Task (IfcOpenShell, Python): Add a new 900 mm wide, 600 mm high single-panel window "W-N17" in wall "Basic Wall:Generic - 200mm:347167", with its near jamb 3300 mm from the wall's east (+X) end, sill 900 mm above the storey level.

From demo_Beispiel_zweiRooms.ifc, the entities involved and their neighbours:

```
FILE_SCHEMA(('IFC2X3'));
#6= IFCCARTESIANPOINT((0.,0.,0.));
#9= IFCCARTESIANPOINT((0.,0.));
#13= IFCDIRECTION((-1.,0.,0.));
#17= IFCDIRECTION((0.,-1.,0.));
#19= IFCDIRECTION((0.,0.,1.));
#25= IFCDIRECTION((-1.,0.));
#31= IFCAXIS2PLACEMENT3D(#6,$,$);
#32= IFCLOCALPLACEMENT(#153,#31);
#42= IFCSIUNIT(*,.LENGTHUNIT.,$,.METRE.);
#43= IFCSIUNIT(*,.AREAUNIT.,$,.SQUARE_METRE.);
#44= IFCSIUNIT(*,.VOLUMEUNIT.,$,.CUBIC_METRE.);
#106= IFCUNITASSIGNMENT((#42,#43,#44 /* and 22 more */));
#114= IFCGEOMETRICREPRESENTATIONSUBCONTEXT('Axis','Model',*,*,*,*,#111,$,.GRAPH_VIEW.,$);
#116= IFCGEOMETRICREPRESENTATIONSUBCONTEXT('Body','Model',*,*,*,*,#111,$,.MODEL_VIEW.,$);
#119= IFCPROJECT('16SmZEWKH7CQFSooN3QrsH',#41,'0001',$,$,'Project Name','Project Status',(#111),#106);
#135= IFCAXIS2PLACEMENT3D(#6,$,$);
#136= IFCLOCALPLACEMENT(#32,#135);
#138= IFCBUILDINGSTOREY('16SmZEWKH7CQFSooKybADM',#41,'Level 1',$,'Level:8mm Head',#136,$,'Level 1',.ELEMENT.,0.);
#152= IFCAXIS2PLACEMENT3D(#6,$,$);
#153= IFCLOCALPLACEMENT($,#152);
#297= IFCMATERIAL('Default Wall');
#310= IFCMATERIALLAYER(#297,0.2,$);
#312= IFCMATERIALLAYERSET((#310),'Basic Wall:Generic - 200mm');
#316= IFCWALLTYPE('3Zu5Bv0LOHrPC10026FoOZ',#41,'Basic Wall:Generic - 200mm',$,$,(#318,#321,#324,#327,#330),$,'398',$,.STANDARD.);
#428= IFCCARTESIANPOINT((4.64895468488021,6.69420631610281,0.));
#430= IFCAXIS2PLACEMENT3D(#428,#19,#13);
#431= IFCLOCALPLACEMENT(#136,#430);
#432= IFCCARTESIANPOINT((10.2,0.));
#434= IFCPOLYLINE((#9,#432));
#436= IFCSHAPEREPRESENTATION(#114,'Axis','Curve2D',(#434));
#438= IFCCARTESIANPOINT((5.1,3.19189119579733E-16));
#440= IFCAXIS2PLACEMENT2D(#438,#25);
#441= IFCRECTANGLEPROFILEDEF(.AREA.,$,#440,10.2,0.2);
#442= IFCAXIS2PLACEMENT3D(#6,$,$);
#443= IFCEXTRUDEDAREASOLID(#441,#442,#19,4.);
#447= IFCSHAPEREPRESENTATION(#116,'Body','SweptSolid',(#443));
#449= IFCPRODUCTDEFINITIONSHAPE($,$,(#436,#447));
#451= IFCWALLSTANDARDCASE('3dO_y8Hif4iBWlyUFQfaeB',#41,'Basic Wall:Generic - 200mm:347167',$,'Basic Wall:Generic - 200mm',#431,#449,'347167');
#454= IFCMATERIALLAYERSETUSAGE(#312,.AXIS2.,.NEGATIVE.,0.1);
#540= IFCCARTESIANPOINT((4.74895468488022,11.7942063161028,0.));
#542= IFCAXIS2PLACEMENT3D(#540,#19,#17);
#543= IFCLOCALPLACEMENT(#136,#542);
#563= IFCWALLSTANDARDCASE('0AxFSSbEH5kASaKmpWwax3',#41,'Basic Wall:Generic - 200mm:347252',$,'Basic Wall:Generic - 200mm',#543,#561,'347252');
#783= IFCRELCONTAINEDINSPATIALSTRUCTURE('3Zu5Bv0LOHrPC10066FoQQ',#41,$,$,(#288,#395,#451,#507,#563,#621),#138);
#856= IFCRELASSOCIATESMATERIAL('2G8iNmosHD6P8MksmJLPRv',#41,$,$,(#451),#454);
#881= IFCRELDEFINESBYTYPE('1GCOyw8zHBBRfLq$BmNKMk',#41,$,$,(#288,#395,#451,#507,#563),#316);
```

```python
import numpy as np
import ifcopenshell
import ifcopenshell.api.feature
import ifcopenshell.api.geometry
import ifcopenshell.api.root
import ifcopenshell.api.spatial
import ifcopenshell.api.type
import ifcopenshell.geom
import ifcopenshell.util.element
import ifcopenshell.util.placement
import ifcopenshell.util.representation
import ifcopenshell.util.shape
import ifcopenshell.util.unit

model = ifcopenshell.open("demo_Beispiel_zweiRooms.ifc")
unit_scale = ifcopenshell.util.unit.calculate_unit_scale(model)
settings = ifcopenshell.geom.settings()


def volume(element):
    """Net volume in cubic metres, openings subtracted."""
    shape = ifcopenshell.geom.create_shape(settings, element)
    return ifcopenshell.util.shape.get_volume(shape.geometry)


wall = model.by_id(451)
storey = ifcopenshell.util.element.get_container(wall, ifc_class="IfcBuildingStorey")
context = ifcopenshell.util.representation.get_context(model, "Model", "Body", "MODEL_VIEW")
before = volume(wall)

width, height, from_end, sill = 0.9, 0.6, 3.3, 0.9  # metres

# The wall runs along its own X axis, and the end named is its -X end.
wall_shape = ifcopenshell.geom.create_shape(settings, wall)
x, y, z = ifcopenshell.util.shape.get_vertices(wall_shape.geometry).T
start = x.min() + from_end
face, thickness = float(y.min()), float(y.max() - y.min())
wall_matrix = ifcopenshell.util.placement.get_local_placement(wall.ObjectPlacement)
level = ifcopenshell.util.placement.get_local_placement(storey.ObjectPlacement)[2, 3]


def in_wall(x, y):
    """Placement at x, y metres in the wall's axes, at sill height."""
    matrix = wall_matrix.copy()
    matrix[:, 3] = wall_matrix @ np.array([x / unit_scale, y / unit_scale, 0.0, 1.0])
    matrix[2, 3] = level + sill / unit_scale
    return matrix


# Opening: a box that overshoots both wall faces by 50 mm.
opening = ifcopenshell.api.root.create_entity(model, ifc_class="IfcOpeningElement")
box = ifcopenshell.api.geometry.add_wall_representation(
    model, context=context, length=width, height=height, thickness=thickness + 0.1
)
ifcopenshell.api.geometry.assign_representation(model, product=opening, representation=box)
ifcopenshell.api.geometry.edit_object_placement(model, product=opening, matrix=in_wall(start, face - 0.05), is_si=False)
ifcopenshell.api.feature.add_feature(model, feature=opening, element=wall)

window = ifcopenshell.api.root.create_entity(model, ifc_class="IfcWindow", name="W-N17")
window.OverallWidth, window.OverallHeight = width / unit_scale, height / unit_scale
body = ifcopenshell.api.geometry.add_window_representation(
    model,
    context=context,
    overall_width=window.OverallWidth,
    overall_height=window.OverallHeight,
    partition_type="SINGLE_PANEL",
)
ifcopenshell.api.geometry.assign_representation(model, product=window, representation=body)
ifcopenshell.api.spatial.assign_container(model, products=[window], relating_structure=storey)
fills = ifcopenshell.api.feature.add_filling(model, opening=opening, element=window)
fills.OwnerHistory = window.OwnerHistory  # required in IFC2X3

# IFC2X3 keeps the operation on the window style.
style = ifcopenshell.api.root.create_entity(model, ifc_class="IfcWindowStyle", name="W-N17")
style.OperationType, style.ConstructionType = "SINGLE_PANEL", "NOTDEFINED"
style.ParameterTakesPrecedence = style.Sizeable = False
ifcopenshell.api.type.assign_type(model, related_objects=[window], relating_type=style)

# Centre the window in the wall's thickness.
ifcopenshell.api.geometry.edit_object_placement(model, product=window, matrix=in_wall(start, face), is_si=False)
window_shape = ifcopenshell.geom.create_shape(settings, window)
depth = ifcopenshell.util.shape.get_vertices(window_shape.geometry)[:, 1]
offset = face + thickness / 2 - (depth.min() + depth.max()) / 2
ifcopenshell.api.geometry.edit_object_placement(model, product=window, matrix=in_wall(start, offset), is_si=False)

after = volume(wall)

print(f"wall volume {before:.3f} -> {after:.3f} m3")

model.write("demo_Beispiel_zweiRooms-out.ifc")
```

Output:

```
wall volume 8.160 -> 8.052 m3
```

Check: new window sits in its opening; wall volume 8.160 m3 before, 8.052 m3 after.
